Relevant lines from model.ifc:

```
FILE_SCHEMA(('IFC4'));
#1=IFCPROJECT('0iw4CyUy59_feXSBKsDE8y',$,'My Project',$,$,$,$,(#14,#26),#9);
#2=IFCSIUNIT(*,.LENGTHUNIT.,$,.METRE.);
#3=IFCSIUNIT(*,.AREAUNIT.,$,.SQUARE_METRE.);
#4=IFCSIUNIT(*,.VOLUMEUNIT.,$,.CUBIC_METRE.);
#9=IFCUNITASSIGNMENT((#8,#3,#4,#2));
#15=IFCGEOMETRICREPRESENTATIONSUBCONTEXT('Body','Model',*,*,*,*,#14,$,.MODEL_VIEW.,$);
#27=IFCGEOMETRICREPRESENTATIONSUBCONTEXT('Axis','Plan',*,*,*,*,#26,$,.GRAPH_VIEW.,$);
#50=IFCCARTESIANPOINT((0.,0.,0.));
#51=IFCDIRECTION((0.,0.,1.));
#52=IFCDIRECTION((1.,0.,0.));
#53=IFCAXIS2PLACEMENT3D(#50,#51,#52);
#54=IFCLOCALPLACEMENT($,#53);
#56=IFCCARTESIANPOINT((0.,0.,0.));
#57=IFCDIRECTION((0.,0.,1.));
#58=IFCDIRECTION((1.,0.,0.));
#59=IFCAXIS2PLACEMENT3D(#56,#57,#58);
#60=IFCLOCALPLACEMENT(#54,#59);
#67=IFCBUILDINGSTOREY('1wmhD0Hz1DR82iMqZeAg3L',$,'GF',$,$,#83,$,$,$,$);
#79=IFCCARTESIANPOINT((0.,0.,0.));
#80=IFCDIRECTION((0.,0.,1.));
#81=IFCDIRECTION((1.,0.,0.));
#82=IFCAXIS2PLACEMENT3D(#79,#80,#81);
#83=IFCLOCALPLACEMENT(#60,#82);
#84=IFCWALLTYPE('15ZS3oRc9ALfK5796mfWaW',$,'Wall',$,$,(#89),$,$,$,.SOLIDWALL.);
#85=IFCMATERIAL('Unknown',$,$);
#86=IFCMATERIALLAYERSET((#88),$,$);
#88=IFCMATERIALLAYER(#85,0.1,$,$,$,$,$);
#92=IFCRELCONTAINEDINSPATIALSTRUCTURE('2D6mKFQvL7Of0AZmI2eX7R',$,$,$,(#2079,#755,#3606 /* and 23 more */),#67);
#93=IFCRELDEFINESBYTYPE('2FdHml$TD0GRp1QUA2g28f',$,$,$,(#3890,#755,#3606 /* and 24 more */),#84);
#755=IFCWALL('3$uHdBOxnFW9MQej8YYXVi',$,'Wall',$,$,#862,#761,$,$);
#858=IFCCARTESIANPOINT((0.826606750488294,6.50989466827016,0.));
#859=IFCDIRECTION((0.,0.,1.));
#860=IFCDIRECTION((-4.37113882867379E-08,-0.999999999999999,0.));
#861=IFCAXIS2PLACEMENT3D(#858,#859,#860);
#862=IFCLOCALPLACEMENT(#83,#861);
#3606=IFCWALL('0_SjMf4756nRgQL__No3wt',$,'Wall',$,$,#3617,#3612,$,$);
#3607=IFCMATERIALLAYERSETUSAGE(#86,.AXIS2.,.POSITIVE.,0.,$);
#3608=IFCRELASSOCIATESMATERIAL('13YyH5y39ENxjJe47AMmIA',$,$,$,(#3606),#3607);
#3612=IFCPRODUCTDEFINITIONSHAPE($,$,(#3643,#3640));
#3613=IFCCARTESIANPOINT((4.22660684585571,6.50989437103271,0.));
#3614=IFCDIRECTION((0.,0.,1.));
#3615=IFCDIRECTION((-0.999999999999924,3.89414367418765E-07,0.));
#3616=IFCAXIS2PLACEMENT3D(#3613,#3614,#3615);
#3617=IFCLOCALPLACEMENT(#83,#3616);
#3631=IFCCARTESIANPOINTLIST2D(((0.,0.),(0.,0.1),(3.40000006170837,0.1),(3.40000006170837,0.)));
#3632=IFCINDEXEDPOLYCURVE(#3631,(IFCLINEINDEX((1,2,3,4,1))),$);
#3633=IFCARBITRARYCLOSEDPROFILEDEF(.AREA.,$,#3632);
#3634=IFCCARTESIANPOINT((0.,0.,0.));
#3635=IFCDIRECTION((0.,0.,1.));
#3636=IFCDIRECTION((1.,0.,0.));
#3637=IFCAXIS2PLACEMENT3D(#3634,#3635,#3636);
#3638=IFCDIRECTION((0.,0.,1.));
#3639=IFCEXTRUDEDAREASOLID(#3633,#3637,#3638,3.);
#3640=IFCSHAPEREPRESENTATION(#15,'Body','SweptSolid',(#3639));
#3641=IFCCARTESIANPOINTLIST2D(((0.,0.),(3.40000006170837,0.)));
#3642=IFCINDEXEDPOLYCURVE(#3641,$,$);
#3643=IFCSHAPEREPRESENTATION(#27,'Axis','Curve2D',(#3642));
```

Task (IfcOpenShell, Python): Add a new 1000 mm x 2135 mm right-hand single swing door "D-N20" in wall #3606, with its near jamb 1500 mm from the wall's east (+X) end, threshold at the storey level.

```python
import numpy as np
import ifcopenshell
import ifcopenshell.api.feature
import ifcopenshell.api.geometry
import ifcopenshell.api.root
import ifcopenshell.api.spatial
import ifcopenshell.geom
import ifcopenshell.util.element
import ifcopenshell.util.placement
import ifcopenshell.util.representation
import ifcopenshell.util.shape
import ifcopenshell.util.unit

model = ifcopenshell.open("model.ifc")
unit_scale = ifcopenshell.util.unit.calculate_unit_scale(model)
settings = ifcopenshell.geom.settings()


def volume(element):
    """Net volume in cubic metres, openings subtracted."""
    shape = ifcopenshell.geom.create_shape(settings, element)
    return ifcopenshell.util.shape.get_volume(shape.geometry)


wall = model.by_guid("0_SjMf4756nRgQL__No3wt")
storey = ifcopenshell.util.element.get_container(wall, ifc_class="IfcBuildingStorey")
context = ifcopenshell.util.representation.get_context(model, "Model", "Body", "MODEL_VIEW")
before = volume(wall)

width, height, from_end, sill = 1, 2.135, 1.5, 0.0  # metres

# The wall runs along its own X axis, and the end named is its -X end.
wall_shape = ifcopenshell.geom.create_shape(settings, wall)
x, y, z = ifcopenshell.util.shape.get_vertices(wall_shape.geometry).T
start = x.min() + from_end
face, thickness = float(y.min()), float(y.max() - y.min())
wall_matrix = ifcopenshell.util.placement.get_local_placement(wall.ObjectPlacement)
level = ifcopenshell.util.placement.get_local_placement(storey.ObjectPlacement)[2, 3]


def in_wall(x, y):
    """Placement at x, y metres in the wall's axes, at sill height."""
    matrix = wall_matrix.copy()
    matrix[:, 3] = wall_matrix @ np.array([x / unit_scale, y / unit_scale, 0.0, 1.0])
    matrix[2, 3] = level + sill / unit_scale
    return matrix


# Opening: a box that overshoots both wall faces by 50 mm.
opening = ifcopenshell.api.root.create_entity(model, ifc_class="IfcOpeningElement", predefined_type="OPENING")
box = ifcopenshell.api.geometry.add_wall_representation(
    model, context=context, length=width, height=height, thickness=thickness + 0.1
)
ifcopenshell.api.geometry.assign_representation(model, product=opening, representation=box)
ifcopenshell.api.geometry.edit_object_placement(model, product=opening, matrix=in_wall(start, face - 0.05), is_si=False)
ifcopenshell.api.feature.add_feature(model, feature=opening, element=wall)

door = ifcopenshell.api.root.create_entity(model, ifc_class="IfcDoor", name="D-N20", predefined_type="DOOR")
door.OverallWidth, door.OverallHeight = width / unit_scale, height / unit_scale
door.OperationType = "SINGLE_SWING_RIGHT"
body = ifcopenshell.api.geometry.add_door_representation(
    model,
    context=context,
    overall_width=door.OverallWidth,
    overall_height=door.OverallHeight,
    operation_type="SINGLE_SWING_RIGHT",
    lining_properties={"LiningDepth": thickness / unit_scale, "ThresholdDepth": thickness / unit_scale},
)
ifcopenshell.api.geometry.assign_representation(model, product=door, representation=body)
ifcopenshell.api.spatial.assign_container(model, products=[door], relating_structure=storey)
ifcopenshell.api.feature.add_filling(model, opening=opening, element=door)

# The lining spans the wall, so the door starts at the wall face.
ifcopenshell.api.geometry.edit_object_placement(model, product=door, matrix=in_wall(start, face), is_si=False)

after = volume(wall)

print(f"wall volume {before:.3f} -> {after:.3f} m3")

model.write("model-out.ifc")
```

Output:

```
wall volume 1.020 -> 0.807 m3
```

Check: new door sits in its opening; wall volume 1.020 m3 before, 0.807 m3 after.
